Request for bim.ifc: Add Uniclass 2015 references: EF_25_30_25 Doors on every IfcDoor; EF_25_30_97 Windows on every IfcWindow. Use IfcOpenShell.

First a look at what the model holds.

```python
import ifcopenshell

model = ifcopenshell.open("bim.ifc")
print(model.schema)
print("classifications:", [c.Name for c in model.by_type("IfcClassification")])
for ifc_class in ("IfcDoor", "IfcRoof", "IfcStair", "IfcWall", "IfcWindow"):
    print(ifc_class, len(model.by_type(ifc_class)))
```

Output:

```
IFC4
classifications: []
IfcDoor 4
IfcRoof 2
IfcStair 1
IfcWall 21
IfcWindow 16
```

```python
import ifcopenshell
import ifcopenshell.api.classification

model = ifcopenshell.open("bim.ifc")

system = ifcopenshell.api.classification.add_classification(model, classification="Uniclass 2015")

codes = {
    "IfcDoor": ("EF_25_30_25", "Doors"),
    "IfcWindow": ("EF_25_30_97", "Windows"),
}
for ifc_class, (code, name) in codes.items():
    products = model.by_type(ifc_class)
    ifcopenshell.api.classification.add_reference(
        model, products=products, classification=system, identification=code, name=name
    )
    print(code, len(products))

model.write("bim_rev.ifc")
```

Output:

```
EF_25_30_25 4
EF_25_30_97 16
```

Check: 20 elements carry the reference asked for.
